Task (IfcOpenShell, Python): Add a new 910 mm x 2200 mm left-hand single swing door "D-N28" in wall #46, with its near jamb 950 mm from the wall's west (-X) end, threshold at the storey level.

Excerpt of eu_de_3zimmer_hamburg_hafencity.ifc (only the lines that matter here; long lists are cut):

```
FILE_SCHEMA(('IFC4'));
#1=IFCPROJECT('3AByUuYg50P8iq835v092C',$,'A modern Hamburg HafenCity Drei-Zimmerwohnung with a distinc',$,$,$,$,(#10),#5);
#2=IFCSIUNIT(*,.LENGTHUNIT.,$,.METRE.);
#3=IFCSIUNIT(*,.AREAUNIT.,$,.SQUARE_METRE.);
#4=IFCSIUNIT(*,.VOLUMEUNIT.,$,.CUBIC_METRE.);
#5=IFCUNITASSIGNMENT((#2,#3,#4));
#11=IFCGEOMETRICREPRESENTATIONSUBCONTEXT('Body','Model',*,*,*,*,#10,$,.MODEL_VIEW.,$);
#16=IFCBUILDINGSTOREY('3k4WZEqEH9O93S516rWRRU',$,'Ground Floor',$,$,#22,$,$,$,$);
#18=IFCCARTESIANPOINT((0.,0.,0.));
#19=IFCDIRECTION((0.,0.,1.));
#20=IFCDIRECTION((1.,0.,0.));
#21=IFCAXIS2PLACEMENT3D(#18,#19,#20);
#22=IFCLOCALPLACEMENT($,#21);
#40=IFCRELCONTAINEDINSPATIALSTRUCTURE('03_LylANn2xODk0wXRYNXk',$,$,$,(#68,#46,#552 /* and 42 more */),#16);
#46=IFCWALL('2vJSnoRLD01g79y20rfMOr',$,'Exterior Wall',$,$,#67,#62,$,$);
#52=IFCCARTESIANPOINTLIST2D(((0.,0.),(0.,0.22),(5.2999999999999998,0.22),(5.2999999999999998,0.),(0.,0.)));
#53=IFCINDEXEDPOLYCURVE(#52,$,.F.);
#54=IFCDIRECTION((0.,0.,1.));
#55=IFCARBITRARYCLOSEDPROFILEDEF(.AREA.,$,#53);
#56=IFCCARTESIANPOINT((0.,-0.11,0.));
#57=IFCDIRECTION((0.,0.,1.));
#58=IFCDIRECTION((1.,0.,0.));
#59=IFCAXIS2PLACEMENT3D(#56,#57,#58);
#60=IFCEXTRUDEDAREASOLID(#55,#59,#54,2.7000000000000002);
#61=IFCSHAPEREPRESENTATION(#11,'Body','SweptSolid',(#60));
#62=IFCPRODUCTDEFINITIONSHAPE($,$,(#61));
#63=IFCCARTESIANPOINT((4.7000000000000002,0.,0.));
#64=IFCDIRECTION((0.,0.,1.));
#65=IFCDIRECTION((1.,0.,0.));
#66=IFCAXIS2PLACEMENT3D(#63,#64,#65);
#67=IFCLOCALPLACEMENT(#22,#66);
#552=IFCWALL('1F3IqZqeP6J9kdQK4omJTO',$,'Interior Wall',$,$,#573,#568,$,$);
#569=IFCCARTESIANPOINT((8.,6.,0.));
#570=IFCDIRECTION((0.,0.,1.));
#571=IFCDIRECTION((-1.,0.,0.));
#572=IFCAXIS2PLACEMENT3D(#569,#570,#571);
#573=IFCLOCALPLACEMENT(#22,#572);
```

```python
import numpy as np
import ifcopenshell
import ifcopenshell.api.feature
import ifcopenshell.api.geometry
import ifcopenshell.api.root
import ifcopenshell.api.spatial
import ifcopenshell.geom
import ifcopenshell.util.element
import ifcopenshell.util.placement
import ifcopenshell.util.representation
import ifcopenshell.util.shape
import ifcopenshell.util.unit

model = ifcopenshell.open("eu_de_3zimmer_hamburg_hafencity.ifc")
unit_scale = ifcopenshell.util.unit.calculate_unit_scale(model)
settings = ifcopenshell.geom.settings()


def volume(element):
    """Net volume in cubic metres, openings subtracted."""
    shape = ifcopenshell.geom.create_shape(settings, element)
    return ifcopenshell.util.shape.get_volume(shape.geometry)


wall = model.by_guid("2vJSnoRLD01g79y20rfMOr")
storey = ifcopenshell.util.element.get_container(wall, ifc_class="IfcBuildingStorey")
context = ifcopenshell.util.representation.get_context(model, "Model", "Body", "MODEL_VIEW")
before = volume(wall)

width, height, from_end, sill = 0.91, 2.2, 0.95, 0.0  # metres

# The wall runs along its own X axis, and the end named is its -X end.
wall_shape = ifcopenshell.geom.create_shape(settings, wall)
x, y, z = ifcopenshell.util.shape.get_vertices(wall_shape.geometry).T
start = x.min() + from_end
face, thickness = float(y.min()), float(y.max() - y.min())
wall_matrix = ifcopenshell.util.placement.get_local_placement(wall.ObjectPlacement)
level = ifcopenshell.util.placement.get_local_placement(storey.ObjectPlacement)[2, 3]


def in_wall(x, y):
    """Placement at x, y metres in the wall's axes, at sill height."""
    matrix = wall_matrix.copy()
    matrix[:, 3] = wall_matrix @ np.array([x / unit_scale, y / unit_scale, 0.0, 1.0])
    matrix[2, 3] = level + sill / unit_scale
    return matrix


# Opening: a box that overshoots both wall faces by 50 mm.
opening = ifcopenshell.api.root.create_entity(model, ifc_class="IfcOpeningElement", predefined_type="OPENING")
box = ifcopenshell.api.geometry.add_wall_representation(
    model, context=context, length=width, height=height, thickness=thickness + 0.1
)
ifcopenshell.api.geometry.assign_representation(model, product=opening, representation=box)
ifcopenshell.api.geometry.edit_object_placement(model, product=opening, matrix=in_wall(start, face - 0.05), is_si=False)
ifcopenshell.api.feature.add_feature(model, feature=opening, element=wall)

door = ifcopenshell.api.root.create_entity(model, ifc_class="IfcDoor", name="D-N28", predefined_type="DOOR")
door.OverallWidth, door.OverallHeight = width / unit_scale, height / unit_scale
door.OperationType = "SINGLE_SWING_LEFT"
body = ifcopenshell.api.geometry.add_door_representation(
    model,
    context=context,
    overall_width=door.OverallWidth,
    overall_height=door.OverallHeight,
    operation_type="SINGLE_SWING_LEFT",
    lining_properties={"LiningDepth": thickness / unit_scale, "ThresholdDepth": thickness / unit_scale},
)
ifcopenshell.api.geometry.assign_representation(model, product=door, representation=body)
ifcopenshell.api.spatial.assign_container(model, products=[door], relating_structure=storey)
ifcopenshell.api.feature.add_filling(model, opening=opening, element=door)

# The lining spans the wall, so the door starts at the wall face.
ifcopenshell.api.geometry.edit_object_placement(model, product=door, matrix=in_wall(start, face), is_si=False)

after = volume(wall)

print(f"wall volume {before:.3f} -> {after:.3f} m3")

model.write("eu_de_3zimmer_hamburg_hafencity_updated.ifc")
```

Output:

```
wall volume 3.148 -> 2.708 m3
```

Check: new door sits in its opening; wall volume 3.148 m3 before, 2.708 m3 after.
